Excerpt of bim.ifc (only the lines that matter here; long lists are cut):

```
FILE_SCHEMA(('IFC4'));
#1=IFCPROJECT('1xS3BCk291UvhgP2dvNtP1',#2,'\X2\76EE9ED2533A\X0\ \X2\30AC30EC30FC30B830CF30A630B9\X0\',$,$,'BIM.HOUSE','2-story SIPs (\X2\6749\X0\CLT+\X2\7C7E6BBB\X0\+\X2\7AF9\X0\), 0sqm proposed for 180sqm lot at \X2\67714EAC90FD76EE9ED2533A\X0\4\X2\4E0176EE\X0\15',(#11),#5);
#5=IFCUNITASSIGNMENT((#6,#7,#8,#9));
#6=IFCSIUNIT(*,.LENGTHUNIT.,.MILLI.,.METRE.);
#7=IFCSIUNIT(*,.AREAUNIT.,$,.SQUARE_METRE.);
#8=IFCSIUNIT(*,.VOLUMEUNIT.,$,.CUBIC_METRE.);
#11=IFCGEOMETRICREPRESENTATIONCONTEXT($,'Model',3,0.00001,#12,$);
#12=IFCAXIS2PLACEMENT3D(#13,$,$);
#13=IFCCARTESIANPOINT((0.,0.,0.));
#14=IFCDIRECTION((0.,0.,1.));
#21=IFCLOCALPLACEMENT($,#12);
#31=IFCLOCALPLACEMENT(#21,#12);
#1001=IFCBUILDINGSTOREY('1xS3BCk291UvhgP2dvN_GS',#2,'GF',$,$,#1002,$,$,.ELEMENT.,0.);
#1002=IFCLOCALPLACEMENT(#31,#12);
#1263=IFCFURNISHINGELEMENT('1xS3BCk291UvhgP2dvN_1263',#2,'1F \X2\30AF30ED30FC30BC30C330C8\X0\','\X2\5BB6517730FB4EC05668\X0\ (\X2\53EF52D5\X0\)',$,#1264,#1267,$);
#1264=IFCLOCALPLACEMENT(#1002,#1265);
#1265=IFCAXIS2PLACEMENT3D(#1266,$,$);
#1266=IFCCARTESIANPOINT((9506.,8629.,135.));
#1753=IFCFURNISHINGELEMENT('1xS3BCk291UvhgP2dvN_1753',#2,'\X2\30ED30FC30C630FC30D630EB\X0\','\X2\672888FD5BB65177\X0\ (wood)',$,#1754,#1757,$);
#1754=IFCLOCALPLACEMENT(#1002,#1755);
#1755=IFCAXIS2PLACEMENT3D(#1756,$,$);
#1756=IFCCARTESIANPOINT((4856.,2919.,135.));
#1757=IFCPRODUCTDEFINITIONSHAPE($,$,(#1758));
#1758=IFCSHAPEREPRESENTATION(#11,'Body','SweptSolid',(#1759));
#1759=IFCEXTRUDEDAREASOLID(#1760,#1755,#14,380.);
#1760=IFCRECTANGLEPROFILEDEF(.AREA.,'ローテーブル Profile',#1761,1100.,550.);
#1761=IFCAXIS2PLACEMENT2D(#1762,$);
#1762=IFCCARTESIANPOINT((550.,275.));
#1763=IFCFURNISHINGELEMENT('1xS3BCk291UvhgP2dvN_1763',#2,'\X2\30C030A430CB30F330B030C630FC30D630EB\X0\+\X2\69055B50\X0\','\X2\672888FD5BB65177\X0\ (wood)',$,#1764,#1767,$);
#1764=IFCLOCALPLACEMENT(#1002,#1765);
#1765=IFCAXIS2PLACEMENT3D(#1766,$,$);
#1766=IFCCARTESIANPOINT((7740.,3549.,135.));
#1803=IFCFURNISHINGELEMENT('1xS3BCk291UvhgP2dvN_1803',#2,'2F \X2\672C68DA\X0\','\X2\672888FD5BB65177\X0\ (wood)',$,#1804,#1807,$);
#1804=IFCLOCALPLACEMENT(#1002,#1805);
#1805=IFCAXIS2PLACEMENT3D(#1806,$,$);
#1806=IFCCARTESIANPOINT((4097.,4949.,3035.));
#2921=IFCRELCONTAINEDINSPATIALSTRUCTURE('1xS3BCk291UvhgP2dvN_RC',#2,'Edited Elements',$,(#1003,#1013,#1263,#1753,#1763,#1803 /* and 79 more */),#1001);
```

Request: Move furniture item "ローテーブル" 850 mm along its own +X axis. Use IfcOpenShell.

```python
import ifcopenshell
import ifcopenshell.api.geometry
import ifcopenshell.util.placement
import ifcopenshell.util.unit

model = ifcopenshell.open("bim.ifc")
unit_scale = ifcopenshell.util.unit.calculate_unit_scale(model)

item = model.by_guid("1xS3BCk291UvhgP2dvN_1753")
matrix = ifcopenshell.util.placement.get_local_placement(item.ObjectPlacement)
matrix[:3, 3] += matrix[:3, 0] * 0.85 / unit_scale
ifcopenshell.api.geometry.edit_object_placement(model, product=item, matrix=matrix, is_si=False)

print(ifcopenshell.util.placement.get_local_placement(item.ObjectPlacement).round(3) + 0.0)

model.write("bim_updated.ifc")
```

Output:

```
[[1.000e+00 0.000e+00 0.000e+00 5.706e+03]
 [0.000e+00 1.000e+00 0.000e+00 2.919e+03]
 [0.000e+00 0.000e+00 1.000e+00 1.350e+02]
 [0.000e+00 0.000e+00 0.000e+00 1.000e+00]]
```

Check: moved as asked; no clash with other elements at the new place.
